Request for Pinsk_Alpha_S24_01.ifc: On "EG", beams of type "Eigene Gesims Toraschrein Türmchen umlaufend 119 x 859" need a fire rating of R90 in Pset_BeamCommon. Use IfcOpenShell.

First a look at what the model holds.

```python
import ifcopenshell
import ifcopenshell.util.element

model = ifcopenshell.open("Pinsk_Alpha_S24_01.ifc")
print(model.schema)
storey = next(s for s in model.by_type("IfcBuildingStorey") if s.Name == "EG")
beams = [e for e in ifcopenshell.util.element.get_decomposition(storey) if e.is_a("IfcBeam")]
seen = {}
for e in beams:
    element_type = ifcopenshell.util.element.get_type(e)
    key = (element_type.Name if element_type != e and element_type else None, ifcopenshell.util.element.get_pset(e, "Pset_BeamCommon", "FireRating"))
    seen[key] = seen.get(key, 0) + 1
for (name, value), count in sorted(seen.items(), key=str):
    print(count, "x", name, "|", value)
```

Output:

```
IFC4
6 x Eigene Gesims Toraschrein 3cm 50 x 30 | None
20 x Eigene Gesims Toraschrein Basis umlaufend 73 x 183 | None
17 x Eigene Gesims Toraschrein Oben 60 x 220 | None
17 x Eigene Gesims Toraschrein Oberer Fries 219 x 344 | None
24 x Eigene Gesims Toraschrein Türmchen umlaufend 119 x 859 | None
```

```python
import ifcopenshell
import ifcopenshell.api.pset
import ifcopenshell.util.element

model = ifcopenshell.open("Pinsk_Alpha_S24_01.ifc")

storey = next(s for s in model.by_type("IfcBuildingStorey") if s.Name == "EG")
beams = [e for e in ifcopenshell.util.element.get_decomposition(storey) if e.is_a("IfcBeam")]

count = 0
for e in beams:
    element_type = ifcopenshell.util.element.get_type(e)
    if element_type in (None, e) or element_type.Name != "Eigene Gesims Toraschrein Türmchen umlaufend 119 x 859":
        continue
    # add_pset returns the element's existing set when there is one.
    pset = ifcopenshell.api.pset.add_pset(model, product=e, name="Pset_BeamCommon")
    ifcopenshell.api.pset.edit_pset(model, pset=pset, properties={"FireRating": "R90"})
    count += 1

print(count, "beams updated")

model.write("Pinsk_Alpha_S24_01_edited.ifc")
```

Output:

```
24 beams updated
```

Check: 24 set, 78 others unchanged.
